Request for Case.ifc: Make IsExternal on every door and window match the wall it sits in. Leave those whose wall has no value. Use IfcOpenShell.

First a look at what the model holds.

```python
import ifcopenshell
import ifcopenshell.util.element

model = ifcopenshell.open("Case.ifc")
print(model.schema)
seen = {}
for e in model.by_type("IfcDoor") + model.by_type("IfcWindow"):
    if not e.FillsVoids:
        continue
    host = e.FillsVoids[0].RelatingOpeningElement.VoidsElements[0].RelatingBuildingElement
    own = ifcopenshell.util.element.get_pset(e, f"Pset_{e.is_a()[3:].removesuffix('StandardCase')}Common", "IsExternal")
    wall = ifcopenshell.util.element.get_pset(host, "Pset_WallCommon", "IsExternal")
    seen[e.is_a(), own, wall] = seen.get((e.is_a(), own, wall), 0) + 1
for (cls, own, wall), count in sorted(seen.items(), key=str):
    print(count, cls, "IsExternal:", own, "| host wall:", wall)
```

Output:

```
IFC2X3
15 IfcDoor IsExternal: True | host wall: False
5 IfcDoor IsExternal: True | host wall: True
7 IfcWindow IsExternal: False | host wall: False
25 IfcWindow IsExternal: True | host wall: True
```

```python
import ifcopenshell
import ifcopenshell.api.pset
import ifcopenshell.util.element

model = ifcopenshell.open("Case.ifc")

count = 0
for ifc_class, pset_name in (("IfcDoor", "Pset_DoorCommon"), ("IfcWindow", "Pset_WindowCommon")):
    for e in model.by_type(ifc_class):
        if not e.FillsVoids:
            continue
        host = e.FillsVoids[0].RelatingOpeningElement.VoidsElements[0].RelatingBuildingElement
        external = ifcopenshell.util.element.get_pset(host, "Pset_WallCommon", "IsExternal")
        if external is None or ifcopenshell.util.element.get_pset(e, pset_name, "IsExternal") == external:
            continue
        pset = ifcopenshell.api.pset.add_pset(model, product=e, name=pset_name)
        ifcopenshell.api.pset.edit_pset(model, pset=pset, properties={"IsExternal": external})
        count += 1

print(count, "updated")

model.write("Case_edited.ifc")
```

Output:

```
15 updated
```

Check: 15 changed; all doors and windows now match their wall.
